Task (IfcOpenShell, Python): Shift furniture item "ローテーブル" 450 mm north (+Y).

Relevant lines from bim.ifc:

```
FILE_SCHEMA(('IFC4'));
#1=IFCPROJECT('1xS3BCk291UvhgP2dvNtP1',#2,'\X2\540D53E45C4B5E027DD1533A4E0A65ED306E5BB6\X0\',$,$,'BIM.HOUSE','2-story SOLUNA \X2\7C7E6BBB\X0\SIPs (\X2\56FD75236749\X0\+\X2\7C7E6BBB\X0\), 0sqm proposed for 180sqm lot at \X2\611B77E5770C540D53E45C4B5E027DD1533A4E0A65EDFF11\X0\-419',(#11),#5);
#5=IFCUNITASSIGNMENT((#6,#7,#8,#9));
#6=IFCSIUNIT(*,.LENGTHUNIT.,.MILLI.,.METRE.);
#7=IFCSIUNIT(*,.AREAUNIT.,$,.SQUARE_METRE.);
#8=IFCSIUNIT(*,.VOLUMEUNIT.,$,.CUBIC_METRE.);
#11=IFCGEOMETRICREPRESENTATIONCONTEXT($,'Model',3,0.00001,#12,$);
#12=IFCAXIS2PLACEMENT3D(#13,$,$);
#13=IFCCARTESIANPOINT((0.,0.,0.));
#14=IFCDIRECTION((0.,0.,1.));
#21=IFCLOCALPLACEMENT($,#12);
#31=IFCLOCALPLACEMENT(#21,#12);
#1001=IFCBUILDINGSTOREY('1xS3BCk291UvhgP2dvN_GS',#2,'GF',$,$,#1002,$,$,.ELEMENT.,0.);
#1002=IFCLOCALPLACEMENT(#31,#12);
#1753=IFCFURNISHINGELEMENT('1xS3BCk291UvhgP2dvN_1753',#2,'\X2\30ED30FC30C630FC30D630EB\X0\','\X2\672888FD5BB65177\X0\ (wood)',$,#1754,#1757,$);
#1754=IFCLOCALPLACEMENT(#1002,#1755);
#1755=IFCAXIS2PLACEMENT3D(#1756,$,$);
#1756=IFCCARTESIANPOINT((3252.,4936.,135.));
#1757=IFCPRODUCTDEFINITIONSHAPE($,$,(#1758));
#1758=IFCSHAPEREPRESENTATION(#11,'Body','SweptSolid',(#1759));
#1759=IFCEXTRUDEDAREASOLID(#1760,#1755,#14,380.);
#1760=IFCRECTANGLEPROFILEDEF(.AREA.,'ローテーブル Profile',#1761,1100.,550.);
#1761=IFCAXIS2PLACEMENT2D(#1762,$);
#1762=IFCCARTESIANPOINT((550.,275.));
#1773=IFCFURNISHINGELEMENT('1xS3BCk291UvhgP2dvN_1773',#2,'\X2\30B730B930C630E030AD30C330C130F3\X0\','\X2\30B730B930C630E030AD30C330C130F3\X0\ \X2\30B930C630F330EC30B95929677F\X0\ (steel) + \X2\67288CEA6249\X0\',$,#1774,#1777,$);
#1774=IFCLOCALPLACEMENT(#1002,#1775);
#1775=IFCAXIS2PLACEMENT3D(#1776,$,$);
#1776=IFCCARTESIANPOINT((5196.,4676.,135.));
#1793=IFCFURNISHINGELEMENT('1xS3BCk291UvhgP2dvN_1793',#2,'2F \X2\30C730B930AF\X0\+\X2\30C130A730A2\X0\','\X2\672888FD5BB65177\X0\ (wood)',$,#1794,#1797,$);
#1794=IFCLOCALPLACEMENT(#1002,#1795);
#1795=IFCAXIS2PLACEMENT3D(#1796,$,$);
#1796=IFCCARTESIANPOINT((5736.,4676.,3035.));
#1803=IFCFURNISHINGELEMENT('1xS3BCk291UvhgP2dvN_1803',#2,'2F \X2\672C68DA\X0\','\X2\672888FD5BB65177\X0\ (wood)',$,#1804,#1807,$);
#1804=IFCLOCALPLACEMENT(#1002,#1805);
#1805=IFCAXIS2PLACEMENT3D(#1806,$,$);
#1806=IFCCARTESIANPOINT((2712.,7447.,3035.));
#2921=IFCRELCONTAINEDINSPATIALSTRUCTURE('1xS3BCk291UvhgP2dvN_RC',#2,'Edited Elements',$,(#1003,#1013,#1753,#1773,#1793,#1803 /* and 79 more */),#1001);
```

```python
import ifcopenshell
import ifcopenshell.api.geometry
import ifcopenshell.util.placement
import ifcopenshell.util.unit

model = ifcopenshell.open("bim.ifc")
unit_scale = ifcopenshell.util.unit.calculate_unit_scale(model)

item = model.by_id(1753)
matrix = ifcopenshell.util.placement.get_local_placement(item.ObjectPlacement)
matrix[1, 3] += 0.45 / unit_scale
ifcopenshell.api.geometry.edit_object_placement(model, product=item, matrix=matrix, is_si=False)

print(ifcopenshell.util.placement.get_local_placement(item.ObjectPlacement).round(3) + 0.0)

model.write("bim_v2.ifc")
```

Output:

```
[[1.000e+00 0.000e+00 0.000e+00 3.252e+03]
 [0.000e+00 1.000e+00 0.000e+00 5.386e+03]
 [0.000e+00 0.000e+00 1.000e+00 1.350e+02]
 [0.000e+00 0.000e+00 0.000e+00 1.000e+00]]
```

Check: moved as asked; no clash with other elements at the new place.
